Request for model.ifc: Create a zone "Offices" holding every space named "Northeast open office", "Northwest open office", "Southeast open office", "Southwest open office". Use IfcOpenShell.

First a look at what the model holds.

```python
import ifcopenshell

model = ifcopenshell.open("model.ifc")
print(model.schema)
seen = {}
for space in model.by_type("IfcSpace"):
    seen[space.LongName] = seen.get(space.LongName, 0) + 1
for name, count in sorted(seen.items(), key=str):
    print(count, "x", name)
print("zones:", [z.Name for z in model.by_type("IfcZone")][:20])
```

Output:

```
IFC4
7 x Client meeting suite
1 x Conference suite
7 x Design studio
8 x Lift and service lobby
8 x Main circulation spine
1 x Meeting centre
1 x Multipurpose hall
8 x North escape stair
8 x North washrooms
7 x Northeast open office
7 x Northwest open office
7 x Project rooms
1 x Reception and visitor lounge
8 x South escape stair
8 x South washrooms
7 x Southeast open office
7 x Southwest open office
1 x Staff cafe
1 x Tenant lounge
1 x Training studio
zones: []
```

```python
import ifcopenshell
import ifcopenshell.api.group
import ifcopenshell.api.root

model = ifcopenshell.open("model.ifc")

names = {"Northeast open office", "Northwest open office", "Southeast open office", "Southwest open office"}
spaces = [s for s in model.by_type("IfcSpace") if s.LongName in names]

zone = ifcopenshell.api.root.create_entity(model, ifc_class="IfcZone", name="Offices")
ifcopenshell.api.group.assign_group(model, products=spaces, group=zone)
print(len(spaces), "spaces in", zone.Name)

model.write("model-out.ifc")
```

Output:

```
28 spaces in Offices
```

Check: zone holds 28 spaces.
